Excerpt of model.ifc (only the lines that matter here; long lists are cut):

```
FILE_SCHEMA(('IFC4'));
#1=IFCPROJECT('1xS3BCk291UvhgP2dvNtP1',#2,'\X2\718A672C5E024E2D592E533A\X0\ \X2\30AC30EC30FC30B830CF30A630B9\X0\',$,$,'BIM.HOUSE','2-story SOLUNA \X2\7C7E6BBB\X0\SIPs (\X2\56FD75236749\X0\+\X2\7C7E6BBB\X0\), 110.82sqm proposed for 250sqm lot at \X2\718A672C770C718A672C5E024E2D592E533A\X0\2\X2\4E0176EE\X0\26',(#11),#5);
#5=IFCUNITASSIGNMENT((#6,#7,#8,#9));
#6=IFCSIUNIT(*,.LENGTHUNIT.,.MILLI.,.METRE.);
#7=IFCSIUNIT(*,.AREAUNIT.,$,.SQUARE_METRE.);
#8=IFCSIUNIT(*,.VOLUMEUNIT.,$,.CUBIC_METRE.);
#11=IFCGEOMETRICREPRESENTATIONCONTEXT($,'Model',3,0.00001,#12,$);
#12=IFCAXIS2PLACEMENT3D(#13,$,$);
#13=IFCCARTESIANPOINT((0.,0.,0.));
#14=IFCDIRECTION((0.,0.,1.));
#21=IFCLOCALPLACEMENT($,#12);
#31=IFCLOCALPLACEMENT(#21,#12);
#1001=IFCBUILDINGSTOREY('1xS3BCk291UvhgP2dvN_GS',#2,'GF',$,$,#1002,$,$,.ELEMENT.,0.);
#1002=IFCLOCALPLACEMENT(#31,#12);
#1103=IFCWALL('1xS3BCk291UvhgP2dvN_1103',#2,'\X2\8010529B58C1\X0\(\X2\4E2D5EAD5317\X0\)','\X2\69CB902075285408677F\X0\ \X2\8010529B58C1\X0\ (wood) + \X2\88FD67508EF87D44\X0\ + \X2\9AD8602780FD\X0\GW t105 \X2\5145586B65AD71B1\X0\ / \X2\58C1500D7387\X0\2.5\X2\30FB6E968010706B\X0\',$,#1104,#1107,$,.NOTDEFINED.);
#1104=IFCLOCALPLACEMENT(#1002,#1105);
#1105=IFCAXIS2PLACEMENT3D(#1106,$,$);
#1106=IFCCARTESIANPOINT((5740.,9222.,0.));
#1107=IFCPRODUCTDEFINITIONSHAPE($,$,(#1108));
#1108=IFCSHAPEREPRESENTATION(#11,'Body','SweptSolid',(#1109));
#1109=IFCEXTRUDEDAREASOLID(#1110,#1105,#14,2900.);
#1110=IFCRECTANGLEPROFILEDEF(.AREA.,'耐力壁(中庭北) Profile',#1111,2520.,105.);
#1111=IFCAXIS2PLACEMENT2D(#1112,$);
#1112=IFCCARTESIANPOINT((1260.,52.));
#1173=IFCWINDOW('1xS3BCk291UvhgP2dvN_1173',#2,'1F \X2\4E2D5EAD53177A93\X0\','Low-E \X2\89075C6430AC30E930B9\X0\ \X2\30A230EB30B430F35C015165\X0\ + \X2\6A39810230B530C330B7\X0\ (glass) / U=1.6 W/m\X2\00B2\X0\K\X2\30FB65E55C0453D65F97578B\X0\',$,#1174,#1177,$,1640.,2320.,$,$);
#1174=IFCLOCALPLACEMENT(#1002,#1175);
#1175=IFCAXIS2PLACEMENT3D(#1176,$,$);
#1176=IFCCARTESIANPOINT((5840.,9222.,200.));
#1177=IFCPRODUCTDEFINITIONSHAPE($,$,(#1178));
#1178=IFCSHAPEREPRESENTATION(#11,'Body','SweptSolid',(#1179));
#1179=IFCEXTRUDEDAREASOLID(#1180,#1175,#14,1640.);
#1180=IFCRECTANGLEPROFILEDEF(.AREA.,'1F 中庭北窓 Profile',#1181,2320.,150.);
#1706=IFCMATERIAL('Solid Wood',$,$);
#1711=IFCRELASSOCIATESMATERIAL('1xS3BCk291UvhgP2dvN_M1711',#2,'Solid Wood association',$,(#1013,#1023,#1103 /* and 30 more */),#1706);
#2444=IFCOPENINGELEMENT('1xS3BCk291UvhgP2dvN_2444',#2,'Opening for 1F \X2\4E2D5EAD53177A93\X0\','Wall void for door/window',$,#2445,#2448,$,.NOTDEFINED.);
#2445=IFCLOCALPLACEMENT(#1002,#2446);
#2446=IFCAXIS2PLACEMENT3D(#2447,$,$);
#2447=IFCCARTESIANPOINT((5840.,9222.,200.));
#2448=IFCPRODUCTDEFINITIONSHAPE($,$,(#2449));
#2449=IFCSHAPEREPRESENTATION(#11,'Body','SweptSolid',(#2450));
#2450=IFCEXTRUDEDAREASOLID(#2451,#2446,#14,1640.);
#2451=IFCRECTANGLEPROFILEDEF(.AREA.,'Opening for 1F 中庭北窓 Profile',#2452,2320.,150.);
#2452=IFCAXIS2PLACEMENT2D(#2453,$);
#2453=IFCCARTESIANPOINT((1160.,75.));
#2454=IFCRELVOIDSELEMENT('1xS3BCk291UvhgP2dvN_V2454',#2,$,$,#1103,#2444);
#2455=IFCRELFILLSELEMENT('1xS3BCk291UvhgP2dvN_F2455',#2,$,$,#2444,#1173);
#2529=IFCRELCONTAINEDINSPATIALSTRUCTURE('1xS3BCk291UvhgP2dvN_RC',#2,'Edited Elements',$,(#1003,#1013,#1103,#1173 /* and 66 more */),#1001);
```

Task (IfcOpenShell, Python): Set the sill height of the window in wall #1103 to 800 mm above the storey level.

```python
import numpy as np
import ifcopenshell
import ifcopenshell.api.geometry
import ifcopenshell.geom
import ifcopenshell.util.element
import ifcopenshell.util.placement
import ifcopenshell.util.shape
import ifcopenshell.util.unit

model = ifcopenshell.open("model.ifc")
unit_scale = ifcopenshell.util.unit.calculate_unit_scale(model)

window = model.by_id(1173)
opening = window.FillsVoids[0].RelatingOpeningElement
storey = ifcopenshell.util.element.get_container(window, ifc_class="IfcBuildingStorey")
level = ifcopenshell.util.placement.get_local_placement(storey.ObjectPlacement)[2, 3]

# The opening's origin need not be at the sill, so measure its lowest point.
shape = ifcopenshell.geom.create_shape(ifcopenshell.geom.settings(), opening)
bottom = ifcopenshell.util.shape.get_shape_bottom_elevation(shape, shape.geometry) / unit_scale
dz = level + 0.8 / unit_scale - bottom

shift = np.array([0.0, 0.0, dz])
# The window is not placed relative to its opening, so move both.
for product in (opening, window):
    matrix = ifcopenshell.util.placement.get_local_placement(product.ObjectPlacement)
    matrix[:3, 3] += shift
    ifcopenshell.api.geometry.edit_object_placement(model, product=product, matrix=matrix, is_si=False)

print(f"moved by {dz * unit_scale:+.3f} m")

model.write("model_updated.ifc")
```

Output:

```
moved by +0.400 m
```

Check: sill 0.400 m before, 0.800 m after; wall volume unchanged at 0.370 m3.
